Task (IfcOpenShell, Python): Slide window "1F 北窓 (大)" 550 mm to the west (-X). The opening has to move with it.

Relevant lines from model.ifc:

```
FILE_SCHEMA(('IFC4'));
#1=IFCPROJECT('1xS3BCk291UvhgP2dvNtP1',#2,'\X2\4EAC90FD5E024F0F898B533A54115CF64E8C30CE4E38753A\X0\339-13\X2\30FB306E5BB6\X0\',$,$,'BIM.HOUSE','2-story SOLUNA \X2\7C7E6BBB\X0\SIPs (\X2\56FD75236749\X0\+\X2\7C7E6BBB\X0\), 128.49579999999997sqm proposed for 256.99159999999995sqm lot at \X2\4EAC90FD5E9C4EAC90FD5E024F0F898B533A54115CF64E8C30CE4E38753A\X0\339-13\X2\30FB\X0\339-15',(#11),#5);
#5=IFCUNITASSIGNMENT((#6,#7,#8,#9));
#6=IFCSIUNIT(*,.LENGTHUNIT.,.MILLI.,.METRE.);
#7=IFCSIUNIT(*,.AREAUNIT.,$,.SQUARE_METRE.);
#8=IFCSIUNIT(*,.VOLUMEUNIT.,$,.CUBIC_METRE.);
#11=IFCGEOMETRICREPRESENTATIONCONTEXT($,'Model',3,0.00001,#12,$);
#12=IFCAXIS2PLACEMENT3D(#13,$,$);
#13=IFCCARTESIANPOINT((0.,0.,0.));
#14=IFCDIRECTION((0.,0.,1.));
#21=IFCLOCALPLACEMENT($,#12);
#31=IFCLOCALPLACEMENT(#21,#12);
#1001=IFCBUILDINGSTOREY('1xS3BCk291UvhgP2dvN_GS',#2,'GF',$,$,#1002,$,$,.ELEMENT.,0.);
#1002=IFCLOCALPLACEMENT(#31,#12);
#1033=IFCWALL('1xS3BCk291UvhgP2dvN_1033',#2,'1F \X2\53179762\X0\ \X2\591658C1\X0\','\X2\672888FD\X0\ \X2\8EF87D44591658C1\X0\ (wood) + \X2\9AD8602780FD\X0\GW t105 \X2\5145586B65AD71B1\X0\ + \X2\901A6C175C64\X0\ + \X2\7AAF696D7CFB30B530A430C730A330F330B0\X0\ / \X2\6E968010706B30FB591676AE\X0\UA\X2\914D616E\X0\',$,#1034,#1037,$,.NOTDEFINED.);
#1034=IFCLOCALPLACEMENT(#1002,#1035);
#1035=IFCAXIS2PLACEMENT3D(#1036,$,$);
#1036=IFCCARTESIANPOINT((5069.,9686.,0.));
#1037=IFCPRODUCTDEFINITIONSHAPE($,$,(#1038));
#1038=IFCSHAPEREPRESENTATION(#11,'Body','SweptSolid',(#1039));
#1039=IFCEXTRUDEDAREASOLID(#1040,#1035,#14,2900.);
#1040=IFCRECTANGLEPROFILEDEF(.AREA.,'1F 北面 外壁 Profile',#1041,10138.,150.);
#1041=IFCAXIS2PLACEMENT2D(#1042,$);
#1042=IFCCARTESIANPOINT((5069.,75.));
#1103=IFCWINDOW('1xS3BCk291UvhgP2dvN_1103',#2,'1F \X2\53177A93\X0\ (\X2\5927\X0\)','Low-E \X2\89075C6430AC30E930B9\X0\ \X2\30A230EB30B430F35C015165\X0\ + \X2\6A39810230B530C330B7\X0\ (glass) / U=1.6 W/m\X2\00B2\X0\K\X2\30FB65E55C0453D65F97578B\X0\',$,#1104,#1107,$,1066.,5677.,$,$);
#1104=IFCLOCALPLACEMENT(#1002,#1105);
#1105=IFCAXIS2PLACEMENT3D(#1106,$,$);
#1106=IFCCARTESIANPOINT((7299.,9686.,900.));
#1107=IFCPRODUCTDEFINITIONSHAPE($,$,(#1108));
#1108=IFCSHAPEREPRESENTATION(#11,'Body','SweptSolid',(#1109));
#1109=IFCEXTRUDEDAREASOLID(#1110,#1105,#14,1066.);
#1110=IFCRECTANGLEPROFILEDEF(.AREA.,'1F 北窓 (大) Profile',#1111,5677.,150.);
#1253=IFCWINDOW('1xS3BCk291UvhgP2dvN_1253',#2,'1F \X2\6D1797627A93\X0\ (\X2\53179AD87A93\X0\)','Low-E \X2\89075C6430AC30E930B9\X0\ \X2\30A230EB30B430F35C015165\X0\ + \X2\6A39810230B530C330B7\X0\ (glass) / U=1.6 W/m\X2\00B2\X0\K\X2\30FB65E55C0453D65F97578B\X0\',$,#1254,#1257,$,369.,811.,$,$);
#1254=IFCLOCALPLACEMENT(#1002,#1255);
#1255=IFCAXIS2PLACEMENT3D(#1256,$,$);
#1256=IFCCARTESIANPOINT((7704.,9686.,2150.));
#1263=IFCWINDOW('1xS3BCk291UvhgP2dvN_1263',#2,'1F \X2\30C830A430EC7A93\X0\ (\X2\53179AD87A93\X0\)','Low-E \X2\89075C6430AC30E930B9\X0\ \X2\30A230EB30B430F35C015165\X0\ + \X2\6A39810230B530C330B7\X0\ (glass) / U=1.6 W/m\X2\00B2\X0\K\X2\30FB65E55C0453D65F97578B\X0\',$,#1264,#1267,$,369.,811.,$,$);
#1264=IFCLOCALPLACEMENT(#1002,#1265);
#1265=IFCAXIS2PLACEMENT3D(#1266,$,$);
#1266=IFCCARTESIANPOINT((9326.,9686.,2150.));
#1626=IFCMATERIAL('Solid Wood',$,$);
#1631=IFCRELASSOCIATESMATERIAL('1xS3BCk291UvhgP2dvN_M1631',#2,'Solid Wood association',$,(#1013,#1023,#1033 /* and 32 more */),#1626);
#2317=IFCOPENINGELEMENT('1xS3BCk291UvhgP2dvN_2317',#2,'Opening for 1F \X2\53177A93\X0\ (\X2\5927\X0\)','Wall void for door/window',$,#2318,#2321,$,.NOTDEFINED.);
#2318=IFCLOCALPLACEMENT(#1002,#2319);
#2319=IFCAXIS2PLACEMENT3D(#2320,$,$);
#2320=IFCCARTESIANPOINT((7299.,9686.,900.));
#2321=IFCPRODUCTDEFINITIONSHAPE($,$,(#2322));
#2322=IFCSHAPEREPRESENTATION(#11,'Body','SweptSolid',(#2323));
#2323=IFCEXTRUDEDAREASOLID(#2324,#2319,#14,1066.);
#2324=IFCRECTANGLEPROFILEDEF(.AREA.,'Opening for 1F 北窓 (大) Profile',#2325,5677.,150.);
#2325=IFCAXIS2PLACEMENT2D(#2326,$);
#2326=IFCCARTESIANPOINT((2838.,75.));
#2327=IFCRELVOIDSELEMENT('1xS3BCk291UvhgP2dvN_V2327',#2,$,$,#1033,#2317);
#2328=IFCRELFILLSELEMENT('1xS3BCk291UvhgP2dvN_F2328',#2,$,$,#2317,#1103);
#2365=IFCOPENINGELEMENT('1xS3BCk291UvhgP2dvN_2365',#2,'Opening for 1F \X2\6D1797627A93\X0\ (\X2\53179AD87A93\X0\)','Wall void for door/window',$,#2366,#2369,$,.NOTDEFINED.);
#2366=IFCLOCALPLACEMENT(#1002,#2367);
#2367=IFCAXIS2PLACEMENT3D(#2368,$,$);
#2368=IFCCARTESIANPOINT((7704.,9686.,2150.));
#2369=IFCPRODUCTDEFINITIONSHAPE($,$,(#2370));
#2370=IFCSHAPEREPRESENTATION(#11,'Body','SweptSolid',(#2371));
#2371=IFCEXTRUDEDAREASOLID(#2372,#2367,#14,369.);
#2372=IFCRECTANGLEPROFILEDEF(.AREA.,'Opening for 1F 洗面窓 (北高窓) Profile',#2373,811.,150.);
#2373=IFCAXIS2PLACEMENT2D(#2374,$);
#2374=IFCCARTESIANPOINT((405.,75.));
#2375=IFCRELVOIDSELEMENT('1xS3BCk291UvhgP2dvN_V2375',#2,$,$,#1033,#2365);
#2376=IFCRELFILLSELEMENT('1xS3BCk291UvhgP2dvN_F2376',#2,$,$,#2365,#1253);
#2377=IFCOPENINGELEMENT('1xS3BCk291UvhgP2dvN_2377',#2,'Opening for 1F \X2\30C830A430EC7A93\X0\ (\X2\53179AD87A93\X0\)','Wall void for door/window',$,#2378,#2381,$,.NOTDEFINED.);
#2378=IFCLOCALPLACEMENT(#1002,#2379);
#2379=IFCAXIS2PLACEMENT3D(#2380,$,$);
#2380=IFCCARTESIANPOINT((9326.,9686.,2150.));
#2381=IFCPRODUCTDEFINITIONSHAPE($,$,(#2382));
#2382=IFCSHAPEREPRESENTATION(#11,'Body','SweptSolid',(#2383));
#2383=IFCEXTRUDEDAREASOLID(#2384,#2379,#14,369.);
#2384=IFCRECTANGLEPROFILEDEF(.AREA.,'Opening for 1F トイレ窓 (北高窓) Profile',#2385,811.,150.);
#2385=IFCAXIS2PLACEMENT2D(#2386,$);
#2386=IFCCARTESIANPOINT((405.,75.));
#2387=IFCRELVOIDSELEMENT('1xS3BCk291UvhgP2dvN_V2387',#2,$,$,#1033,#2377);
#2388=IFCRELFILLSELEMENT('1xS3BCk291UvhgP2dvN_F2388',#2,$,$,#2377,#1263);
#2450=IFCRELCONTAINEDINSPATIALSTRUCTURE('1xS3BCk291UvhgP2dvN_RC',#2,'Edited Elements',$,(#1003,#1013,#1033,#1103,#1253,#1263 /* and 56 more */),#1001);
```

```python
import ifcopenshell
import ifcopenshell.api.geometry
import ifcopenshell.util.placement

model = ifcopenshell.open("model.ifc")

window = model.by_guid("1xS3BCk291UvhgP2dvN_1103")
opening = window.FillsVoids[0].RelatingOpeningElement
wall = opening.VoidsElements[0].RelatingBuildingElement

wall_matrix = ifcopenshell.util.placement.get_local_placement(wall.ObjectPlacement)
shift = wall_matrix[:3, 0] * -550.0
before = ifcopenshell.util.placement.get_local_placement(window.ObjectPlacement)[:3, 3].copy()

# The window is not placed relative to its opening, so move both.
for product in (opening, window):
    matrix = ifcopenshell.util.placement.get_local_placement(product.ObjectPlacement)
    matrix[:3, 3] += shift
    ifcopenshell.api.geometry.edit_object_placement(model, product=product, matrix=matrix, is_si=False)

after = ifcopenshell.util.placement.get_local_placement(window.ObjectPlacement)[:3, 3]
print("window moved by", (after - before).round(3) + 0.0)

model.write("model_updated.ifc")
```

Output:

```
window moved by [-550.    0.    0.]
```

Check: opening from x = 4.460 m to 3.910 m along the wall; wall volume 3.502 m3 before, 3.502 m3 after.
